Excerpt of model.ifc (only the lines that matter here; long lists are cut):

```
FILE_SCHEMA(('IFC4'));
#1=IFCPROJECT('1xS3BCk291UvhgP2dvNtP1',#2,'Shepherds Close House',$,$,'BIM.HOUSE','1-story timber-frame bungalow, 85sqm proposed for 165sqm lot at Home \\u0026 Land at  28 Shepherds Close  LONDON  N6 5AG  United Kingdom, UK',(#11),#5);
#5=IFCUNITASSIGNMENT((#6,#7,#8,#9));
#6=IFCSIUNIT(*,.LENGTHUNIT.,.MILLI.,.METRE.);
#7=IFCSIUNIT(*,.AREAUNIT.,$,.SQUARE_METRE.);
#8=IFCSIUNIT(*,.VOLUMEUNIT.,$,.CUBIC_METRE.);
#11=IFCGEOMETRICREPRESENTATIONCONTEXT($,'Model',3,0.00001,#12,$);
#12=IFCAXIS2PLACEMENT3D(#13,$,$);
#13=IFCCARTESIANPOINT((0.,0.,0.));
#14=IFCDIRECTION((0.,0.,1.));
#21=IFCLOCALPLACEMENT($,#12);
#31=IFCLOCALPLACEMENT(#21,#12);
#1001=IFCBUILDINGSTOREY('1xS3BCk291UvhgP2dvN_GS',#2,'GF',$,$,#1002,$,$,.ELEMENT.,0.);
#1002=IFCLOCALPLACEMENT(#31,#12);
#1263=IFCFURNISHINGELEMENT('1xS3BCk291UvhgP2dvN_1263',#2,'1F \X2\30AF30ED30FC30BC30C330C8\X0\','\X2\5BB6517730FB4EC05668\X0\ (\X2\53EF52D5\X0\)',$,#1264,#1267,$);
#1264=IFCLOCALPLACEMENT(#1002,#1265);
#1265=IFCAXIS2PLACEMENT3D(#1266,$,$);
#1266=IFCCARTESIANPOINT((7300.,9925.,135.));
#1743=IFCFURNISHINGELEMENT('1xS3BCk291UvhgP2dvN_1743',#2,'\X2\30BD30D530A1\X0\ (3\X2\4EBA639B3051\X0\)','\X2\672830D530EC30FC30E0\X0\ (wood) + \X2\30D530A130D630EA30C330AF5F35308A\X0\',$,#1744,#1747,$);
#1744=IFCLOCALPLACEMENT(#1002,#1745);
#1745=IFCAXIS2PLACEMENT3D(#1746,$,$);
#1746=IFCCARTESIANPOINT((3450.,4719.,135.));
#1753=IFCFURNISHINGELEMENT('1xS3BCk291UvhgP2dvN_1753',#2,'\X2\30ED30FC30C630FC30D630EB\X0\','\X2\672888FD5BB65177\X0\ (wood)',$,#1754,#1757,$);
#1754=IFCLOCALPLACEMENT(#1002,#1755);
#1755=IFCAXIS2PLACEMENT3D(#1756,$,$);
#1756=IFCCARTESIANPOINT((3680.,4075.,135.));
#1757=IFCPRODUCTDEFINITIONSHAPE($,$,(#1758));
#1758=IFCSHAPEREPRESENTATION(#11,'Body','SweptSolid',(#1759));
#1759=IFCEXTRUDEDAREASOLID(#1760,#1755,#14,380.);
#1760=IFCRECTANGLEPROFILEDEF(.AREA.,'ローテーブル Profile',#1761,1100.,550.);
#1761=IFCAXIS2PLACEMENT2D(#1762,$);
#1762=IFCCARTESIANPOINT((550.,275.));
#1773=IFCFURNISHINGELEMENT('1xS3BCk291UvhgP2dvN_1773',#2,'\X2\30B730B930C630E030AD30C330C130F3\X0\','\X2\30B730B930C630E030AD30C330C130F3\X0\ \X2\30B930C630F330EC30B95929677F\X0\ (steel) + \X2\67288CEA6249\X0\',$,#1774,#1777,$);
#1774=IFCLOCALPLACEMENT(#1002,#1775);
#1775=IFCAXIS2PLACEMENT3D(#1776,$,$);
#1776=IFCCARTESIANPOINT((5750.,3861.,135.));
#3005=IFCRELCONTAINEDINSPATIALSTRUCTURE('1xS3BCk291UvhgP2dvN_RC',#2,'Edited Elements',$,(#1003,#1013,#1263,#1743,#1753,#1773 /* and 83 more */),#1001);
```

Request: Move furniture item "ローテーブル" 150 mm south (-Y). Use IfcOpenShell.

```python
import ifcopenshell
import ifcopenshell.api.geometry
import ifcopenshell.util.placement

model = ifcopenshell.open("model.ifc")

item = model.by_guid("1xS3BCk291UvhgP2dvN_1753")
matrix = ifcopenshell.util.placement.get_local_placement(item.ObjectPlacement)
matrix[1, 3] -= 150.0
ifcopenshell.api.geometry.edit_object_placement(model, product=item, matrix=matrix, is_si=False)

print(ifcopenshell.util.placement.get_local_placement(item.ObjectPlacement).round(3) + 0.0)

model.write("model_rev.ifc")
```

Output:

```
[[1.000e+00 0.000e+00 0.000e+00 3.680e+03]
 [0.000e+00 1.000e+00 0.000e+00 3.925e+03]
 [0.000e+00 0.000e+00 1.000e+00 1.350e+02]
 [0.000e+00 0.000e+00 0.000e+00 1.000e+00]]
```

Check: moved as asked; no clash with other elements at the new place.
